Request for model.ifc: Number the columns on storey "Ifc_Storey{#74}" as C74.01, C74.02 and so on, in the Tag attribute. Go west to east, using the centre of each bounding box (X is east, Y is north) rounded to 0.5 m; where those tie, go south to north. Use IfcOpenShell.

First a look at what the model holds.

```python
import ifcopenshell
import ifcopenshell.util.element
import ifcopenshell.util.placement

model = ifcopenshell.open("model.ifc")
print(model.schema)
storey = next(s for s in model.by_type("IfcBuildingStorey") if s.Name == "Ifc_Storey{#74}")
columns = [e for e in ifcopenshell.util.element.get_decomposition(storey) if e.is_a("IfcColumn")]
for e in sorted(columns, key=lambda e: e.id()):
    origin = ifcopenshell.util.placement.get_local_placement(e.ObjectPlacement)[:3, 3]
    print(e.id(), e.Tag, e.Name, origin.round(2) + 0.0, sep=" | ")
```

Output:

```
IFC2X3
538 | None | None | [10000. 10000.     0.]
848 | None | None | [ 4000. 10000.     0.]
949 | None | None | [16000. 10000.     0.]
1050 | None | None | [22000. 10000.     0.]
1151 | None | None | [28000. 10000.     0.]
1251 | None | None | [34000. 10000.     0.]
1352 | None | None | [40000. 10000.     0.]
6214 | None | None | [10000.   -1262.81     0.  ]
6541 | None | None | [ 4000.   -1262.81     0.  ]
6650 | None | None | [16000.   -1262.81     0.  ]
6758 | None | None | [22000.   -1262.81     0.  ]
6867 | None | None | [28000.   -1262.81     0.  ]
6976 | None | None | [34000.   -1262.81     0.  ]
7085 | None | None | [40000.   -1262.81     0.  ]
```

```python
import ifcopenshell
import ifcopenshell.geom
import ifcopenshell.util.element
import ifcopenshell.util.shape

model = ifcopenshell.open("model.ifc")
settings = ifcopenshell.geom.settings()
settings.set("use-world-coords", True)


def centre(element):
    shape = ifcopenshell.geom.create_shape(settings, element)
    return ifcopenshell.util.shape.get_bbox_centroid(shape.geometry)


storey = next(s for s in model.by_type("IfcBuildingStorey") if s.Name == "Ifc_Storey{#74}")
columns = [e for e in ifcopenshell.util.element.get_decomposition(storey) if e.is_a("IfcColumn")]

# Insertion points can sit at a corner or the storey origin, so sort by the geometry (in metres).
centres = {e: centre(e) for e in columns}
columns.sort(key=lambda e: (round(centres[e][0] / 0.5), centres[e][1]))

for i, e in enumerate(columns, start=1):
    number = f"C74.{i:02d}"
    e.Tag = number
    print(e.id(), number)

model.write("model-out.ifc")
```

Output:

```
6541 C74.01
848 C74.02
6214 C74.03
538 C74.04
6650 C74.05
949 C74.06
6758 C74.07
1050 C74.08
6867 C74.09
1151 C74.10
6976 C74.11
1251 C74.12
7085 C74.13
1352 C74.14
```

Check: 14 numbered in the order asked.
